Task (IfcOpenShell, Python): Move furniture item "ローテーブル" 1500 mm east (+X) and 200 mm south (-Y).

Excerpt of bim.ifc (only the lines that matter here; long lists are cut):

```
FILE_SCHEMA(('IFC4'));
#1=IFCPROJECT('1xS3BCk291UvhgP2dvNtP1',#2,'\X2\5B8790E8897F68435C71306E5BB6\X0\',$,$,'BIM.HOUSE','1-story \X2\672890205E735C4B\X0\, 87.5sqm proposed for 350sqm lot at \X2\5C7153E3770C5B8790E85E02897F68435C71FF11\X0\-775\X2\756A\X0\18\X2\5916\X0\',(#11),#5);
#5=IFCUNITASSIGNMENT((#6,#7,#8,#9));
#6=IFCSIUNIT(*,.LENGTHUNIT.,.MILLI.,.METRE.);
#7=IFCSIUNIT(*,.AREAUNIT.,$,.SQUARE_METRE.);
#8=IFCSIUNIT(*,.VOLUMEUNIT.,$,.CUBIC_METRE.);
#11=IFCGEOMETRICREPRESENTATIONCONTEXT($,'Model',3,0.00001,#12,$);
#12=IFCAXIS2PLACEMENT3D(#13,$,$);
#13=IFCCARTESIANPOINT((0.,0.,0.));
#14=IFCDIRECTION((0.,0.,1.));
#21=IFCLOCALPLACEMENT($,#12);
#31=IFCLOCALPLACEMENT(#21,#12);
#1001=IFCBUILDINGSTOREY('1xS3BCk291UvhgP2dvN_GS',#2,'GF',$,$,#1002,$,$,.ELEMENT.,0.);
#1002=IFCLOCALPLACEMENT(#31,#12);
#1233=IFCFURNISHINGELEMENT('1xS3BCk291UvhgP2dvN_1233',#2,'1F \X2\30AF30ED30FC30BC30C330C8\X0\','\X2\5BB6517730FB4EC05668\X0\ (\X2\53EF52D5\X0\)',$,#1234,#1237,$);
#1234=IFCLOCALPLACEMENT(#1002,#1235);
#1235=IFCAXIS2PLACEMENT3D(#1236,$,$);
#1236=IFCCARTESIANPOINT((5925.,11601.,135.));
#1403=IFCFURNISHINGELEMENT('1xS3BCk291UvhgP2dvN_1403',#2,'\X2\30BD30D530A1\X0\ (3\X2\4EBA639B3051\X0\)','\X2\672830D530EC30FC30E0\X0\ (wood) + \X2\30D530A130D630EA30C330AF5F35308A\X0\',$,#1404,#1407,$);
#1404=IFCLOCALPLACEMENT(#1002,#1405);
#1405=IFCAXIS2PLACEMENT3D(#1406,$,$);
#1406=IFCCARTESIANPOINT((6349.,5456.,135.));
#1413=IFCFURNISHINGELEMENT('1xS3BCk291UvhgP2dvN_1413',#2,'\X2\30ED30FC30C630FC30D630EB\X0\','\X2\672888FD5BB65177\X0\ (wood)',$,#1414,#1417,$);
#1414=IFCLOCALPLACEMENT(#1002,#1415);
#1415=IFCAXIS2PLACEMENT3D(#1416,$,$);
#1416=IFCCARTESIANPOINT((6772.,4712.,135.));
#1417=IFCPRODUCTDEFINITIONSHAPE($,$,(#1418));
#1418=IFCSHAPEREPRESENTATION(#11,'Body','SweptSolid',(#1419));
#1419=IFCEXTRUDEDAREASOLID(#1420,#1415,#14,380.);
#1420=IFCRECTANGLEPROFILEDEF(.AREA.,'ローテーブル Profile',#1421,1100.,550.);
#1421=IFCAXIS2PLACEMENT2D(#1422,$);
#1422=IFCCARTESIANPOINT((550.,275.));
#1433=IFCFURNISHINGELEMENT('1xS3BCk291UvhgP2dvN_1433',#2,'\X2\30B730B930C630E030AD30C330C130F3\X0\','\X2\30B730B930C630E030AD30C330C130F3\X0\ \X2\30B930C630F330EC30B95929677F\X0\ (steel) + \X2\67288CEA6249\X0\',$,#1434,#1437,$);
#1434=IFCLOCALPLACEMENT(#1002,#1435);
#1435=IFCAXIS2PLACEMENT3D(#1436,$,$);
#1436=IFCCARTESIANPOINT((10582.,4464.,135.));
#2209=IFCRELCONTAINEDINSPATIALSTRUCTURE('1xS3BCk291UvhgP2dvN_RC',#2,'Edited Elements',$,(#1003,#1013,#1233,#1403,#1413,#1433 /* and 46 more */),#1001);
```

```python
import ifcopenshell
import ifcopenshell.api.geometry
import ifcopenshell.util.placement
import ifcopenshell.util.unit

model = ifcopenshell.open("bim.ifc")
unit_scale = ifcopenshell.util.unit.calculate_unit_scale(model)

item = model.by_guid("1xS3BCk291UvhgP2dvN_1413")
matrix = ifcopenshell.util.placement.get_local_placement(item.ObjectPlacement)
matrix[0, 3] += 1.5 / unit_scale
matrix[1, 3] -= 0.2 / unit_scale
ifcopenshell.api.geometry.edit_object_placement(model, product=item, matrix=matrix, is_si=False)

print(ifcopenshell.util.placement.get_local_placement(item.ObjectPlacement).round(3) + 0.0)

model.write("bim_v2.ifc")
```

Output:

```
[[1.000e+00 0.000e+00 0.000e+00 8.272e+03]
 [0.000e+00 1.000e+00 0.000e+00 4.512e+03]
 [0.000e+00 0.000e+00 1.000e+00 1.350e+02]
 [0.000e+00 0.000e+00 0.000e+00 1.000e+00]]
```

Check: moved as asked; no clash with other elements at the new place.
